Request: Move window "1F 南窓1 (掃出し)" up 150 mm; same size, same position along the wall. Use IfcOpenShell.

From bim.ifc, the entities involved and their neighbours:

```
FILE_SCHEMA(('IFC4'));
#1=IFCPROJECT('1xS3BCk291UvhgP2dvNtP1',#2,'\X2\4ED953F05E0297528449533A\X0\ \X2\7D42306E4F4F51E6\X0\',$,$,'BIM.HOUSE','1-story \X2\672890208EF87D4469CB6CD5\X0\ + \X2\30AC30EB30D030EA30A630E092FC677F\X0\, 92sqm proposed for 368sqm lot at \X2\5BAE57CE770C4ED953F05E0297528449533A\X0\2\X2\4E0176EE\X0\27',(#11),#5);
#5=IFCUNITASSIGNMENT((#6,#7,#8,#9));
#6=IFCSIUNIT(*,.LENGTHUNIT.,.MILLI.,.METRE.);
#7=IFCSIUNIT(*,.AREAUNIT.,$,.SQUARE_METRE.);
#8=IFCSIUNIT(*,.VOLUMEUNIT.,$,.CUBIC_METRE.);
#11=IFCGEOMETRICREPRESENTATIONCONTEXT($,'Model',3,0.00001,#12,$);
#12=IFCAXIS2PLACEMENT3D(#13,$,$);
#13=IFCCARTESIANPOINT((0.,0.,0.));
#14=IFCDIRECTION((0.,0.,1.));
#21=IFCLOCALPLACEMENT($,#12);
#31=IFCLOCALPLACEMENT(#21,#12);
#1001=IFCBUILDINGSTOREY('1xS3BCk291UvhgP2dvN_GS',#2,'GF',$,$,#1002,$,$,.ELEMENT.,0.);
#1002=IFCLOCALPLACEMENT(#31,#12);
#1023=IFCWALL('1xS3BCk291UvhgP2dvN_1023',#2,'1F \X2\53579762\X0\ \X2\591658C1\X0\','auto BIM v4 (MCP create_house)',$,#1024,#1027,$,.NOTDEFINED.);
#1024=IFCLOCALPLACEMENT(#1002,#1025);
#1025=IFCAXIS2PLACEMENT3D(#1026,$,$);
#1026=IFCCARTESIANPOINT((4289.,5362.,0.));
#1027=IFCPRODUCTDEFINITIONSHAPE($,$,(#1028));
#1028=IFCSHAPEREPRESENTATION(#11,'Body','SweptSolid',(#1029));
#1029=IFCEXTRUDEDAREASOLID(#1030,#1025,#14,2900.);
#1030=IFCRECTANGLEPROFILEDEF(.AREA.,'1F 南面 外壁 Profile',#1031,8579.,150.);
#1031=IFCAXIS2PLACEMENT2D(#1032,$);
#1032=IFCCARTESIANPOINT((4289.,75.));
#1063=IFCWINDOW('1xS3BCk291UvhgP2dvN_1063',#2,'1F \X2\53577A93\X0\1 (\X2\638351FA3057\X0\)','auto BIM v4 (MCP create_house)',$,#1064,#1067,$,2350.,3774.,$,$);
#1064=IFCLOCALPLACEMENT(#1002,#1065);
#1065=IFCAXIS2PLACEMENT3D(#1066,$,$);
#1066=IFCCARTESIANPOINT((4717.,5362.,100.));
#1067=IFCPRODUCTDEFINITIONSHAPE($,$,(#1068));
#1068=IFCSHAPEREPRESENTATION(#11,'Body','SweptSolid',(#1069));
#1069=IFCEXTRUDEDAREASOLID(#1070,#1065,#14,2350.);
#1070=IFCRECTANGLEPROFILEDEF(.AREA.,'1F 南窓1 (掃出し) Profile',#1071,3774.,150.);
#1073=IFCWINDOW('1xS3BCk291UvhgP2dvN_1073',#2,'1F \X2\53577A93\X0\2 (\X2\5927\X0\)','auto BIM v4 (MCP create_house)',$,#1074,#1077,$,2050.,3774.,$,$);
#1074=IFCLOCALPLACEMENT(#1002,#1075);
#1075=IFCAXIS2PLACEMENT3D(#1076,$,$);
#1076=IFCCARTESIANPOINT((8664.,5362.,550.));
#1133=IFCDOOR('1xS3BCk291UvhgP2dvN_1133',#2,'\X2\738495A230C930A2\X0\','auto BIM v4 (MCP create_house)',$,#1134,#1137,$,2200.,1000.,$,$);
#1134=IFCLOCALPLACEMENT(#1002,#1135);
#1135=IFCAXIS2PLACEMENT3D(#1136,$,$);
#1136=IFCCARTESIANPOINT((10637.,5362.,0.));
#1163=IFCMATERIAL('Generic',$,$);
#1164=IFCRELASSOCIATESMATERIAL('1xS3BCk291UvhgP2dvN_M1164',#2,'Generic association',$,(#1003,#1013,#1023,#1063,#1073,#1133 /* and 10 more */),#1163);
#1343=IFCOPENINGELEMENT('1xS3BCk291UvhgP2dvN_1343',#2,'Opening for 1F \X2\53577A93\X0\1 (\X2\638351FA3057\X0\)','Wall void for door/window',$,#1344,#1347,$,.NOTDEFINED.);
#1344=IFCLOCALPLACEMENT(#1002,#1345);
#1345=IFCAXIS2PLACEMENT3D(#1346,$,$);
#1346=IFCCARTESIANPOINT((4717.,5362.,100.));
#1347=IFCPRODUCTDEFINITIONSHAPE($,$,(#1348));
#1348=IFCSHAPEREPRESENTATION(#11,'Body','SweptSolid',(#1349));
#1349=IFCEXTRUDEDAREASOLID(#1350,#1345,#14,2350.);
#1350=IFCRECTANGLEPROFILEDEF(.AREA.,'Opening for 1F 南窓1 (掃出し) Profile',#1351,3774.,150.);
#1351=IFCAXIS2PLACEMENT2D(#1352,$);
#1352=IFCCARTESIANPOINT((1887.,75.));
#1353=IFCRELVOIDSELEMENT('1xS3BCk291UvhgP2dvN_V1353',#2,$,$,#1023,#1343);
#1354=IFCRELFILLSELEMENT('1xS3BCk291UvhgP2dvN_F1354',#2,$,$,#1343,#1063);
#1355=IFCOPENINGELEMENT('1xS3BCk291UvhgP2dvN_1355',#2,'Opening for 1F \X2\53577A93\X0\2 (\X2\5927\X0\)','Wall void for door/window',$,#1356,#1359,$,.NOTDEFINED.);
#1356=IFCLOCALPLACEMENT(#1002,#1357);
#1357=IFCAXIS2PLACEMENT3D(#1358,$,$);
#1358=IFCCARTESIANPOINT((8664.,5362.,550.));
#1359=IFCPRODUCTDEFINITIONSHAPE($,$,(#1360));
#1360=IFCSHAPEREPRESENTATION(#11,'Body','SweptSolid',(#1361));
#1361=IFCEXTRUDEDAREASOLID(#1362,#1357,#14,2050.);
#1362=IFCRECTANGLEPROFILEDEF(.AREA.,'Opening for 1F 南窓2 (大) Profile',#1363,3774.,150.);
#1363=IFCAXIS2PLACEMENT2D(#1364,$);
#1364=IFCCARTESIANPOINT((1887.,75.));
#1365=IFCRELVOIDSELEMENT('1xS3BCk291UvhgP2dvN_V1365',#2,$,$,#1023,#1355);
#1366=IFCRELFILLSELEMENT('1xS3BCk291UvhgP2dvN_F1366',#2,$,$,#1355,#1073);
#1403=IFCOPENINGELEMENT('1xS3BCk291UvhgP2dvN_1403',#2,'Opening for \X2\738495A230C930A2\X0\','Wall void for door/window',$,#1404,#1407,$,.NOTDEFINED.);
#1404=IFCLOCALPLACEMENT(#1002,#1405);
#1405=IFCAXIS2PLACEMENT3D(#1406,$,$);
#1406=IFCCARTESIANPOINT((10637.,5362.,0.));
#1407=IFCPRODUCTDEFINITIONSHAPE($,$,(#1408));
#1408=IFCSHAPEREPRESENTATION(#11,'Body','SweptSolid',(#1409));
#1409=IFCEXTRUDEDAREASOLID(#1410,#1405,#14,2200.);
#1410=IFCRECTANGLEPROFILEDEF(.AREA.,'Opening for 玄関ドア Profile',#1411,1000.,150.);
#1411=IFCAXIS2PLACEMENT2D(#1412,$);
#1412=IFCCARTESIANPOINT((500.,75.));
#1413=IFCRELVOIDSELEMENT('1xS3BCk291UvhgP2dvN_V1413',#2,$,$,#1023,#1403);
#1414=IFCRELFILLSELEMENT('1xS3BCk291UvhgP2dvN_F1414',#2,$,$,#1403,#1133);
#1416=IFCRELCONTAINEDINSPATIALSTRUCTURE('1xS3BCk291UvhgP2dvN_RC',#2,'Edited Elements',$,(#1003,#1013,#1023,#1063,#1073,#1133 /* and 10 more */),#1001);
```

```python
import numpy as np
import ifcopenshell
import ifcopenshell.api.geometry
import ifcopenshell.util.placement
import ifcopenshell.util.unit

model = ifcopenshell.open("bim.ifc")
unit_scale = ifcopenshell.util.unit.calculate_unit_scale(model)

window = model.by_guid("1xS3BCk291UvhgP2dvN_1063")
opening = window.FillsVoids[0].RelatingOpeningElement
dz = 150.0

shift = np.array([0.0, 0.0, dz])
# The window is not placed relative to its opening, so move both.
for product in (opening, window):
    matrix = ifcopenshell.util.placement.get_local_placement(product.ObjectPlacement)
    matrix[:3, 3] += shift
    ifcopenshell.api.geometry.edit_object_placement(model, product=product, matrix=matrix, is_si=False)

print(f"moved by {dz * unit_scale:+.3f} m")

model.write("bim_edited.ifc")
```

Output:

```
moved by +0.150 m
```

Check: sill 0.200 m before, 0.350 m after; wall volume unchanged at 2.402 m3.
